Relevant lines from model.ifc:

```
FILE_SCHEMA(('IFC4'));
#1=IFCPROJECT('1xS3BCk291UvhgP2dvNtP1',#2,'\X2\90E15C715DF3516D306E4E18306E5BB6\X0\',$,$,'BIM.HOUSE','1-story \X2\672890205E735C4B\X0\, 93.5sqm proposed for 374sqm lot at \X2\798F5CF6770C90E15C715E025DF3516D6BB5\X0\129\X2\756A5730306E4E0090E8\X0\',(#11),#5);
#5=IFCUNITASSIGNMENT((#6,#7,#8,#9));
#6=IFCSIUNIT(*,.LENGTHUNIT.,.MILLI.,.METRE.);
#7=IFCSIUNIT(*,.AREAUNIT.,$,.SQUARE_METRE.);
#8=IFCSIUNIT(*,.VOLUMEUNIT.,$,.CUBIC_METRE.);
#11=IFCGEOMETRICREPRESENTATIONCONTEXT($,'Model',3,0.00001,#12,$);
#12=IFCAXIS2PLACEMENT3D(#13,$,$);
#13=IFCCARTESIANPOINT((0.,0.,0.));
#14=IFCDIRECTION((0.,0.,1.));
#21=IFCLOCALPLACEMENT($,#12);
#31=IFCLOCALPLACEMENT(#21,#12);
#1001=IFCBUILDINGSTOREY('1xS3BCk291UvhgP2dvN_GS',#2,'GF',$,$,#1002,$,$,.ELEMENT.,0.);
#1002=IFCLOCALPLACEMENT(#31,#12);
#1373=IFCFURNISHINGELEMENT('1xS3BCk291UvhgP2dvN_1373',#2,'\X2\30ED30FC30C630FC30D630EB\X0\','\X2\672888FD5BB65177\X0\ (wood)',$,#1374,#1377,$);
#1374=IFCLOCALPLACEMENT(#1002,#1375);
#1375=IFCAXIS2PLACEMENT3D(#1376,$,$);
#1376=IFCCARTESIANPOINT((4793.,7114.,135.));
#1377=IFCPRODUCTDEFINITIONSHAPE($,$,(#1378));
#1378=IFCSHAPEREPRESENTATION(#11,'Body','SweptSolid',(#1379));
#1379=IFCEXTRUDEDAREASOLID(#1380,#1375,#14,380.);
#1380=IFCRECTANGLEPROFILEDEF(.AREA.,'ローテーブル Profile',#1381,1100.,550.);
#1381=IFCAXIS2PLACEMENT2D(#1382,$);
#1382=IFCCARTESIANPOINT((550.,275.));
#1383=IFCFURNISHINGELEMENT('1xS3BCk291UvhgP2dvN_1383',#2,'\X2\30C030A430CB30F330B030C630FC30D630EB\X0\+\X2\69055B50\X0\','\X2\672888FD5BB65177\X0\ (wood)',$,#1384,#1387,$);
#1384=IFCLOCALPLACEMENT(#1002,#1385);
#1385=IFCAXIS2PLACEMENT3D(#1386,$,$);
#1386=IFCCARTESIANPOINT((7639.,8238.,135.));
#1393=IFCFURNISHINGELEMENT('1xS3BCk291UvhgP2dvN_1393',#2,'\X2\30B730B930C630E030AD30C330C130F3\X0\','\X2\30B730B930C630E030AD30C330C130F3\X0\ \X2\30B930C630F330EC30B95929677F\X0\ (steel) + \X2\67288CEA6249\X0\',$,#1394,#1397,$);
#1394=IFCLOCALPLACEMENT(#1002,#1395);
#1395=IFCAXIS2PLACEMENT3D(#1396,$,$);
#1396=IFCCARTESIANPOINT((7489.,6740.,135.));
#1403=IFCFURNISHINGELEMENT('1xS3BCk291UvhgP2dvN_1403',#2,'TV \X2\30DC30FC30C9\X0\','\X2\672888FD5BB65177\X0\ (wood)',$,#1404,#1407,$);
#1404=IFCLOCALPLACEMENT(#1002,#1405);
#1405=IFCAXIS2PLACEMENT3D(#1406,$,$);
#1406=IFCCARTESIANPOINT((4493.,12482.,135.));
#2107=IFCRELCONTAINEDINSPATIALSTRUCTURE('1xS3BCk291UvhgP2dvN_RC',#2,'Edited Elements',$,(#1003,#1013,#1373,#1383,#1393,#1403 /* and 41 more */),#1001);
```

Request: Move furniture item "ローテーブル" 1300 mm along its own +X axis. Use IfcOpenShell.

```python
import ifcopenshell
import ifcopenshell.api.geometry
import ifcopenshell.util.placement
import ifcopenshell.util.unit

model = ifcopenshell.open("model.ifc")
unit_scale = ifcopenshell.util.unit.calculate_unit_scale(model)

item = model.by_guid("1xS3BCk291UvhgP2dvN_1373")
matrix = ifcopenshell.util.placement.get_local_placement(item.ObjectPlacement)
matrix[:3, 3] += matrix[:3, 0] * 1.3 / unit_scale
ifcopenshell.api.geometry.edit_object_placement(model, product=item, matrix=matrix, is_si=False)

print(ifcopenshell.util.placement.get_local_placement(item.ObjectPlacement).round(3) + 0.0)

model.write("model_rev.ifc")
```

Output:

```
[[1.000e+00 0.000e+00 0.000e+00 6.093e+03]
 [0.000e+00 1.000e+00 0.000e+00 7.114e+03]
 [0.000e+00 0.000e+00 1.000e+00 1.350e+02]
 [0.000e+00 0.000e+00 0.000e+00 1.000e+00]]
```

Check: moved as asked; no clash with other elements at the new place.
